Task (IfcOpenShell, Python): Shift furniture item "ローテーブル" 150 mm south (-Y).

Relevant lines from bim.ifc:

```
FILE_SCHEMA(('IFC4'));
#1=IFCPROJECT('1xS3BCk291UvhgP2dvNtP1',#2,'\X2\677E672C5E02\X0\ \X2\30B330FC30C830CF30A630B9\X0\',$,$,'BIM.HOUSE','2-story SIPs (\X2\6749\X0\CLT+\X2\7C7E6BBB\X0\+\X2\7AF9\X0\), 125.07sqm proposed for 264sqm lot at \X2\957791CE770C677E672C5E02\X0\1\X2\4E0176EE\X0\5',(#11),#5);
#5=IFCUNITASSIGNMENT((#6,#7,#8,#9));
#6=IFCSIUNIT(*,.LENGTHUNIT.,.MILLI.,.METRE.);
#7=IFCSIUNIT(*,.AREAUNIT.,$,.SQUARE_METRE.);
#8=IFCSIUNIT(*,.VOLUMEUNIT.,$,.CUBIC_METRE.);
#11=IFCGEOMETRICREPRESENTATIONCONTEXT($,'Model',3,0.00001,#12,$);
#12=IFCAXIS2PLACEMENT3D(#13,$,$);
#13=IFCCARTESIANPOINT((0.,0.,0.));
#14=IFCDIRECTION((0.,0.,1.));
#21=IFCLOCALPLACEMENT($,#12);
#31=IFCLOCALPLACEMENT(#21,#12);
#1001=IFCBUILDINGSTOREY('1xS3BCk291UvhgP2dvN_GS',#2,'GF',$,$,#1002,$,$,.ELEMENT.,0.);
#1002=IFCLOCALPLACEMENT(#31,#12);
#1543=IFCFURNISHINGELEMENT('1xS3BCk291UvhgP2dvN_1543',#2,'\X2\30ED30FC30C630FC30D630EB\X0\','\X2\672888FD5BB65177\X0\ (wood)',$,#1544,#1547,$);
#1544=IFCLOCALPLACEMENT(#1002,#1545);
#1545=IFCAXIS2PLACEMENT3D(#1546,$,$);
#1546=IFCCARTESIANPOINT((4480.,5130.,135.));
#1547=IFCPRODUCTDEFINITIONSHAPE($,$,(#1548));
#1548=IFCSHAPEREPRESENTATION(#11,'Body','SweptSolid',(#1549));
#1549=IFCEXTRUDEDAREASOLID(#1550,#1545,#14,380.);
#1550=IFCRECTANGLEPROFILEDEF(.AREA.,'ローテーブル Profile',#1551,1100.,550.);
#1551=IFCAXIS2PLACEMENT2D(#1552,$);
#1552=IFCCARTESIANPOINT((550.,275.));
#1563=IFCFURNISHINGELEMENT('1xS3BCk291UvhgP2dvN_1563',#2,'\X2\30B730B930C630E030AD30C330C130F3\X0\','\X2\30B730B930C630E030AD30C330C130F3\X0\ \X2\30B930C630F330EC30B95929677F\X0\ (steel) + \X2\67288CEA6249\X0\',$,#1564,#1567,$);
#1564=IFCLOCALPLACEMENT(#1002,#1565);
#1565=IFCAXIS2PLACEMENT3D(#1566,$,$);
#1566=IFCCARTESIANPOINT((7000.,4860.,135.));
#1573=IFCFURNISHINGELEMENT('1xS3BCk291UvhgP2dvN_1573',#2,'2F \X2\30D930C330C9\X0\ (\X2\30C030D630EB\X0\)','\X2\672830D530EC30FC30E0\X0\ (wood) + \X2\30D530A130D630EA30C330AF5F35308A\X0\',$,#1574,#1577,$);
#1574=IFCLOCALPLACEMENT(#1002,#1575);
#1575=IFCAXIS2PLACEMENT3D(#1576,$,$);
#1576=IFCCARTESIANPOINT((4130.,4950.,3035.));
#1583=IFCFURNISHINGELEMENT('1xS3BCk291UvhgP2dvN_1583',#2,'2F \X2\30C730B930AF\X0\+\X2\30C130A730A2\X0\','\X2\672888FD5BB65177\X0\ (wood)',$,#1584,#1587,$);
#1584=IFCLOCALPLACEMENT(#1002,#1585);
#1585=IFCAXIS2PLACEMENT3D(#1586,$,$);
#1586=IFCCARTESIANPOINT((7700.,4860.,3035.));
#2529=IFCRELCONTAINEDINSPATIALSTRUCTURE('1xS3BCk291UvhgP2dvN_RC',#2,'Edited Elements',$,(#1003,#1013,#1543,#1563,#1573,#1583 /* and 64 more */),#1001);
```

```python
import ifcopenshell
import ifcopenshell.api.geometry
import ifcopenshell.util.placement
import ifcopenshell.util.unit

model = ifcopenshell.open("bim.ifc")
unit_scale = ifcopenshell.util.unit.calculate_unit_scale(model)

item = model.by_guid("1xS3BCk291UvhgP2dvN_1543")
matrix = ifcopenshell.util.placement.get_local_placement(item.ObjectPlacement)
matrix[1, 3] -= 0.15 / unit_scale
ifcopenshell.api.geometry.edit_object_placement(model, product=item, matrix=matrix, is_si=False)

print(ifcopenshell.util.placement.get_local_placement(item.ObjectPlacement).round(3) + 0.0)

model.write("bim_rev.ifc")
```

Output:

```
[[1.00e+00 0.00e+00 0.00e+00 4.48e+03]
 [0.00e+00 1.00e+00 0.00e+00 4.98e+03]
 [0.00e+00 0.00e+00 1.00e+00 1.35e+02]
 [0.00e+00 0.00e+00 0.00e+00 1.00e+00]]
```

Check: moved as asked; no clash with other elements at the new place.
